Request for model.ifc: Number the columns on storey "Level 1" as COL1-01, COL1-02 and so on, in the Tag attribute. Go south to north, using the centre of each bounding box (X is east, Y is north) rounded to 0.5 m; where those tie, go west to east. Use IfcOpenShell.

First a look at what the model holds.

```python
import ifcopenshell
import ifcopenshell.util.element
import ifcopenshell.util.placement

model = ifcopenshell.open("model.ifc")
print(model.schema)
storey = next(s for s in model.by_type("IfcBuildingStorey") if s.Name == "Level 1")
columns = [e for e in ifcopenshell.util.element.get_decomposition(storey) if e.is_a("IfcColumn")]
for e in sorted(columns, key=lambda e: e.id()):
    origin = ifcopenshell.util.placement.get_local_placement(e.ObjectPlacement)[:3, 3]
    print(e.id(), e.Tag, e.Name, origin.round(2) + 0.0, sep=" | ")
```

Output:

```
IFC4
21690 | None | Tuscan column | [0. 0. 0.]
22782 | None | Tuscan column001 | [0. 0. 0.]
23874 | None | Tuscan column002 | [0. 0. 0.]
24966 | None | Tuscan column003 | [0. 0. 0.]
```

```python
import ifcopenshell
import ifcopenshell.geom
import ifcopenshell.util.element
import ifcopenshell.util.shape

model = ifcopenshell.open("model.ifc")
settings = ifcopenshell.geom.settings()
settings.set("use-world-coords", True)


def centre(element):
    shape = ifcopenshell.geom.create_shape(settings, element)
    return ifcopenshell.util.shape.get_bbox_centroid(shape.geometry)


storey = next(s for s in model.by_type("IfcBuildingStorey") if s.Name == "Level 1")
columns = [e for e in ifcopenshell.util.element.get_decomposition(storey) if e.is_a("IfcColumn")]

# Insertion points can sit at a corner or the storey origin, so sort by the geometry (in metres).
centres = {e: centre(e) for e in columns}
columns.sort(key=lambda e: (round(centres[e][1] / 0.5), centres[e][0]))

for i, e in enumerate(columns, start=1):
    number = f"COL1-{i:02d}"
    e.Tag = number
    print(e.id(), number)

model.write("model-out.ifc")
```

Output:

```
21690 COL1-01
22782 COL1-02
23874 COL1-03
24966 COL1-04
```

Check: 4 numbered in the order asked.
